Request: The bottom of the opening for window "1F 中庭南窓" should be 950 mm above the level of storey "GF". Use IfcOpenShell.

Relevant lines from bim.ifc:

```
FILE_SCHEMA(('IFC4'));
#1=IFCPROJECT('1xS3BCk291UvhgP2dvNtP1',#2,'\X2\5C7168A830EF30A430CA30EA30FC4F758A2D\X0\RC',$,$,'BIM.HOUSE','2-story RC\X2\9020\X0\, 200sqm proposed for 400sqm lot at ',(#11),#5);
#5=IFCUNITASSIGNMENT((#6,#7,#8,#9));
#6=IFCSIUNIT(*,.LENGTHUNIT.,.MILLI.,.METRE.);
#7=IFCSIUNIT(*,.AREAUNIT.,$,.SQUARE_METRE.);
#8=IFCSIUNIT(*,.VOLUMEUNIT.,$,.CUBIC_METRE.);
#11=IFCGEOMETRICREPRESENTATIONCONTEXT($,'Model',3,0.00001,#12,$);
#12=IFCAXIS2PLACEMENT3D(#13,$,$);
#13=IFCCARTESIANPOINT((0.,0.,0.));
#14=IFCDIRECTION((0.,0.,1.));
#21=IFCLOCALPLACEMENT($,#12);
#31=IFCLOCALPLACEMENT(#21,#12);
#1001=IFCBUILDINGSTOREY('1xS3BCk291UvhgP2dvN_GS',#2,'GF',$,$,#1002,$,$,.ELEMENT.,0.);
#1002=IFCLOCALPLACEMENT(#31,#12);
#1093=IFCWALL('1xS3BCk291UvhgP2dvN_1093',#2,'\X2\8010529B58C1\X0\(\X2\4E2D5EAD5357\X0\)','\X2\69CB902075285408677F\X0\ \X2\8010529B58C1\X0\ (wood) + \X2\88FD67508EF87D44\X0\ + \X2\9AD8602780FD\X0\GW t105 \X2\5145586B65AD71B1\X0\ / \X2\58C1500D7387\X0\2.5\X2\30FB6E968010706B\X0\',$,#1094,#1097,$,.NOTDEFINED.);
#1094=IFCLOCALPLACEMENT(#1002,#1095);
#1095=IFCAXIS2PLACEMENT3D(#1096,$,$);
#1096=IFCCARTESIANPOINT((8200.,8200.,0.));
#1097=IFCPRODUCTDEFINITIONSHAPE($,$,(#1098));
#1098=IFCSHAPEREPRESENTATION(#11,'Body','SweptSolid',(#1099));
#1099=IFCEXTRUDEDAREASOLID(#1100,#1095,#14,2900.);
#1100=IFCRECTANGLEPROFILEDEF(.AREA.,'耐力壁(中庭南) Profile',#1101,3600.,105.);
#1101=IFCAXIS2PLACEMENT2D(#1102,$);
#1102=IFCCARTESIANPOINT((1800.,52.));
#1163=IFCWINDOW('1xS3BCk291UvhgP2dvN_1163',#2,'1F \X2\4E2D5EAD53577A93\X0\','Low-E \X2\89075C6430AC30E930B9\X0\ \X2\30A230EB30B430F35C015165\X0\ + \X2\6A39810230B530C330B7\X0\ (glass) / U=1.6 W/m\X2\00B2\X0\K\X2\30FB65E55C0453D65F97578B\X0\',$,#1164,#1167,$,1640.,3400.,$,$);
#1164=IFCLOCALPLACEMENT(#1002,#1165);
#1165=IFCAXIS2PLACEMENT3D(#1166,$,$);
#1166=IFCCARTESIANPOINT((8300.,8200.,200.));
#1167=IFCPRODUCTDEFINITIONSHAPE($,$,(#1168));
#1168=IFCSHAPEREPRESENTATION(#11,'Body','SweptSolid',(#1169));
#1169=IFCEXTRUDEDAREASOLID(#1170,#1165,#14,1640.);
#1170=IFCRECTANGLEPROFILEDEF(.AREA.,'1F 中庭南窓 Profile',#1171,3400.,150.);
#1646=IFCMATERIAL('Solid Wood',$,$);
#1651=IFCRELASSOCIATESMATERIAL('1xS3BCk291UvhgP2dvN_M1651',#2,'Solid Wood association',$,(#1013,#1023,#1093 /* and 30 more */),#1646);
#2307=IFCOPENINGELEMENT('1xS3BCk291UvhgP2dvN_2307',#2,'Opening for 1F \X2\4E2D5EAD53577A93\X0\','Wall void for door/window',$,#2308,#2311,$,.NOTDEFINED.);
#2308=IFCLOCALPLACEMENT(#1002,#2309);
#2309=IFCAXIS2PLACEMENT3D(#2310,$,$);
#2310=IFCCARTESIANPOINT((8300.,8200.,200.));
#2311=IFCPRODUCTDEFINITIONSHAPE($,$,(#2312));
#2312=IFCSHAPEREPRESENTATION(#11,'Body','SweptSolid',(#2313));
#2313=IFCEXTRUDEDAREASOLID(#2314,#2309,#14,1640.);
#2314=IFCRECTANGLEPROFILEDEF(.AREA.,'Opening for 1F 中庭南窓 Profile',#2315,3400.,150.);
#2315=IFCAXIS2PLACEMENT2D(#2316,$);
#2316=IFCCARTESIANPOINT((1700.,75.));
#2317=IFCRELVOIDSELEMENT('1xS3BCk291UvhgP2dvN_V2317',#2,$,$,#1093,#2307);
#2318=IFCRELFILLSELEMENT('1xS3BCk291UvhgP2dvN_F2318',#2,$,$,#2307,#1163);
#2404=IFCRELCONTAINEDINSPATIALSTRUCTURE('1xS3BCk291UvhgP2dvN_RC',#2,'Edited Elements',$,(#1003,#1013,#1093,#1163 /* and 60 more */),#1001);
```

```python
import numpy as np
import ifcopenshell
import ifcopenshell.api.geometry
import ifcopenshell.geom
import ifcopenshell.util.element
import ifcopenshell.util.placement
import ifcopenshell.util.shape
import ifcopenshell.util.unit

model = ifcopenshell.open("bim.ifc")
unit_scale = ifcopenshell.util.unit.calculate_unit_scale(model)

window = model.by_guid("1xS3BCk291UvhgP2dvN_1163")
opening = window.FillsVoids[0].RelatingOpeningElement
storey = ifcopenshell.util.element.get_container(window, ifc_class="IfcBuildingStorey")
level = ifcopenshell.util.placement.get_local_placement(storey.ObjectPlacement)[2, 3]

# The opening's origin need not be at the sill, so measure its lowest point.
shape = ifcopenshell.geom.create_shape(ifcopenshell.geom.settings(), opening)
bottom = ifcopenshell.util.shape.get_shape_bottom_elevation(shape, shape.geometry) / unit_scale
dz = level + 950.0 - bottom

shift = np.array([0.0, 0.0, dz])
# The window is not placed relative to its opening, so move both.
for product in (opening, window):
    matrix = ifcopenshell.util.placement.get_local_placement(product.ObjectPlacement)
    matrix[:3, 3] += shift
    ifcopenshell.api.geometry.edit_object_placement(model, product=product, matrix=matrix, is_si=False)

print(f"moved by {dz * unit_scale:+.3f} m")

model.write("bim_edited.ifc")
```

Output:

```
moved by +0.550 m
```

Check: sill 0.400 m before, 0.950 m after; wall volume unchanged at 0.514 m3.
